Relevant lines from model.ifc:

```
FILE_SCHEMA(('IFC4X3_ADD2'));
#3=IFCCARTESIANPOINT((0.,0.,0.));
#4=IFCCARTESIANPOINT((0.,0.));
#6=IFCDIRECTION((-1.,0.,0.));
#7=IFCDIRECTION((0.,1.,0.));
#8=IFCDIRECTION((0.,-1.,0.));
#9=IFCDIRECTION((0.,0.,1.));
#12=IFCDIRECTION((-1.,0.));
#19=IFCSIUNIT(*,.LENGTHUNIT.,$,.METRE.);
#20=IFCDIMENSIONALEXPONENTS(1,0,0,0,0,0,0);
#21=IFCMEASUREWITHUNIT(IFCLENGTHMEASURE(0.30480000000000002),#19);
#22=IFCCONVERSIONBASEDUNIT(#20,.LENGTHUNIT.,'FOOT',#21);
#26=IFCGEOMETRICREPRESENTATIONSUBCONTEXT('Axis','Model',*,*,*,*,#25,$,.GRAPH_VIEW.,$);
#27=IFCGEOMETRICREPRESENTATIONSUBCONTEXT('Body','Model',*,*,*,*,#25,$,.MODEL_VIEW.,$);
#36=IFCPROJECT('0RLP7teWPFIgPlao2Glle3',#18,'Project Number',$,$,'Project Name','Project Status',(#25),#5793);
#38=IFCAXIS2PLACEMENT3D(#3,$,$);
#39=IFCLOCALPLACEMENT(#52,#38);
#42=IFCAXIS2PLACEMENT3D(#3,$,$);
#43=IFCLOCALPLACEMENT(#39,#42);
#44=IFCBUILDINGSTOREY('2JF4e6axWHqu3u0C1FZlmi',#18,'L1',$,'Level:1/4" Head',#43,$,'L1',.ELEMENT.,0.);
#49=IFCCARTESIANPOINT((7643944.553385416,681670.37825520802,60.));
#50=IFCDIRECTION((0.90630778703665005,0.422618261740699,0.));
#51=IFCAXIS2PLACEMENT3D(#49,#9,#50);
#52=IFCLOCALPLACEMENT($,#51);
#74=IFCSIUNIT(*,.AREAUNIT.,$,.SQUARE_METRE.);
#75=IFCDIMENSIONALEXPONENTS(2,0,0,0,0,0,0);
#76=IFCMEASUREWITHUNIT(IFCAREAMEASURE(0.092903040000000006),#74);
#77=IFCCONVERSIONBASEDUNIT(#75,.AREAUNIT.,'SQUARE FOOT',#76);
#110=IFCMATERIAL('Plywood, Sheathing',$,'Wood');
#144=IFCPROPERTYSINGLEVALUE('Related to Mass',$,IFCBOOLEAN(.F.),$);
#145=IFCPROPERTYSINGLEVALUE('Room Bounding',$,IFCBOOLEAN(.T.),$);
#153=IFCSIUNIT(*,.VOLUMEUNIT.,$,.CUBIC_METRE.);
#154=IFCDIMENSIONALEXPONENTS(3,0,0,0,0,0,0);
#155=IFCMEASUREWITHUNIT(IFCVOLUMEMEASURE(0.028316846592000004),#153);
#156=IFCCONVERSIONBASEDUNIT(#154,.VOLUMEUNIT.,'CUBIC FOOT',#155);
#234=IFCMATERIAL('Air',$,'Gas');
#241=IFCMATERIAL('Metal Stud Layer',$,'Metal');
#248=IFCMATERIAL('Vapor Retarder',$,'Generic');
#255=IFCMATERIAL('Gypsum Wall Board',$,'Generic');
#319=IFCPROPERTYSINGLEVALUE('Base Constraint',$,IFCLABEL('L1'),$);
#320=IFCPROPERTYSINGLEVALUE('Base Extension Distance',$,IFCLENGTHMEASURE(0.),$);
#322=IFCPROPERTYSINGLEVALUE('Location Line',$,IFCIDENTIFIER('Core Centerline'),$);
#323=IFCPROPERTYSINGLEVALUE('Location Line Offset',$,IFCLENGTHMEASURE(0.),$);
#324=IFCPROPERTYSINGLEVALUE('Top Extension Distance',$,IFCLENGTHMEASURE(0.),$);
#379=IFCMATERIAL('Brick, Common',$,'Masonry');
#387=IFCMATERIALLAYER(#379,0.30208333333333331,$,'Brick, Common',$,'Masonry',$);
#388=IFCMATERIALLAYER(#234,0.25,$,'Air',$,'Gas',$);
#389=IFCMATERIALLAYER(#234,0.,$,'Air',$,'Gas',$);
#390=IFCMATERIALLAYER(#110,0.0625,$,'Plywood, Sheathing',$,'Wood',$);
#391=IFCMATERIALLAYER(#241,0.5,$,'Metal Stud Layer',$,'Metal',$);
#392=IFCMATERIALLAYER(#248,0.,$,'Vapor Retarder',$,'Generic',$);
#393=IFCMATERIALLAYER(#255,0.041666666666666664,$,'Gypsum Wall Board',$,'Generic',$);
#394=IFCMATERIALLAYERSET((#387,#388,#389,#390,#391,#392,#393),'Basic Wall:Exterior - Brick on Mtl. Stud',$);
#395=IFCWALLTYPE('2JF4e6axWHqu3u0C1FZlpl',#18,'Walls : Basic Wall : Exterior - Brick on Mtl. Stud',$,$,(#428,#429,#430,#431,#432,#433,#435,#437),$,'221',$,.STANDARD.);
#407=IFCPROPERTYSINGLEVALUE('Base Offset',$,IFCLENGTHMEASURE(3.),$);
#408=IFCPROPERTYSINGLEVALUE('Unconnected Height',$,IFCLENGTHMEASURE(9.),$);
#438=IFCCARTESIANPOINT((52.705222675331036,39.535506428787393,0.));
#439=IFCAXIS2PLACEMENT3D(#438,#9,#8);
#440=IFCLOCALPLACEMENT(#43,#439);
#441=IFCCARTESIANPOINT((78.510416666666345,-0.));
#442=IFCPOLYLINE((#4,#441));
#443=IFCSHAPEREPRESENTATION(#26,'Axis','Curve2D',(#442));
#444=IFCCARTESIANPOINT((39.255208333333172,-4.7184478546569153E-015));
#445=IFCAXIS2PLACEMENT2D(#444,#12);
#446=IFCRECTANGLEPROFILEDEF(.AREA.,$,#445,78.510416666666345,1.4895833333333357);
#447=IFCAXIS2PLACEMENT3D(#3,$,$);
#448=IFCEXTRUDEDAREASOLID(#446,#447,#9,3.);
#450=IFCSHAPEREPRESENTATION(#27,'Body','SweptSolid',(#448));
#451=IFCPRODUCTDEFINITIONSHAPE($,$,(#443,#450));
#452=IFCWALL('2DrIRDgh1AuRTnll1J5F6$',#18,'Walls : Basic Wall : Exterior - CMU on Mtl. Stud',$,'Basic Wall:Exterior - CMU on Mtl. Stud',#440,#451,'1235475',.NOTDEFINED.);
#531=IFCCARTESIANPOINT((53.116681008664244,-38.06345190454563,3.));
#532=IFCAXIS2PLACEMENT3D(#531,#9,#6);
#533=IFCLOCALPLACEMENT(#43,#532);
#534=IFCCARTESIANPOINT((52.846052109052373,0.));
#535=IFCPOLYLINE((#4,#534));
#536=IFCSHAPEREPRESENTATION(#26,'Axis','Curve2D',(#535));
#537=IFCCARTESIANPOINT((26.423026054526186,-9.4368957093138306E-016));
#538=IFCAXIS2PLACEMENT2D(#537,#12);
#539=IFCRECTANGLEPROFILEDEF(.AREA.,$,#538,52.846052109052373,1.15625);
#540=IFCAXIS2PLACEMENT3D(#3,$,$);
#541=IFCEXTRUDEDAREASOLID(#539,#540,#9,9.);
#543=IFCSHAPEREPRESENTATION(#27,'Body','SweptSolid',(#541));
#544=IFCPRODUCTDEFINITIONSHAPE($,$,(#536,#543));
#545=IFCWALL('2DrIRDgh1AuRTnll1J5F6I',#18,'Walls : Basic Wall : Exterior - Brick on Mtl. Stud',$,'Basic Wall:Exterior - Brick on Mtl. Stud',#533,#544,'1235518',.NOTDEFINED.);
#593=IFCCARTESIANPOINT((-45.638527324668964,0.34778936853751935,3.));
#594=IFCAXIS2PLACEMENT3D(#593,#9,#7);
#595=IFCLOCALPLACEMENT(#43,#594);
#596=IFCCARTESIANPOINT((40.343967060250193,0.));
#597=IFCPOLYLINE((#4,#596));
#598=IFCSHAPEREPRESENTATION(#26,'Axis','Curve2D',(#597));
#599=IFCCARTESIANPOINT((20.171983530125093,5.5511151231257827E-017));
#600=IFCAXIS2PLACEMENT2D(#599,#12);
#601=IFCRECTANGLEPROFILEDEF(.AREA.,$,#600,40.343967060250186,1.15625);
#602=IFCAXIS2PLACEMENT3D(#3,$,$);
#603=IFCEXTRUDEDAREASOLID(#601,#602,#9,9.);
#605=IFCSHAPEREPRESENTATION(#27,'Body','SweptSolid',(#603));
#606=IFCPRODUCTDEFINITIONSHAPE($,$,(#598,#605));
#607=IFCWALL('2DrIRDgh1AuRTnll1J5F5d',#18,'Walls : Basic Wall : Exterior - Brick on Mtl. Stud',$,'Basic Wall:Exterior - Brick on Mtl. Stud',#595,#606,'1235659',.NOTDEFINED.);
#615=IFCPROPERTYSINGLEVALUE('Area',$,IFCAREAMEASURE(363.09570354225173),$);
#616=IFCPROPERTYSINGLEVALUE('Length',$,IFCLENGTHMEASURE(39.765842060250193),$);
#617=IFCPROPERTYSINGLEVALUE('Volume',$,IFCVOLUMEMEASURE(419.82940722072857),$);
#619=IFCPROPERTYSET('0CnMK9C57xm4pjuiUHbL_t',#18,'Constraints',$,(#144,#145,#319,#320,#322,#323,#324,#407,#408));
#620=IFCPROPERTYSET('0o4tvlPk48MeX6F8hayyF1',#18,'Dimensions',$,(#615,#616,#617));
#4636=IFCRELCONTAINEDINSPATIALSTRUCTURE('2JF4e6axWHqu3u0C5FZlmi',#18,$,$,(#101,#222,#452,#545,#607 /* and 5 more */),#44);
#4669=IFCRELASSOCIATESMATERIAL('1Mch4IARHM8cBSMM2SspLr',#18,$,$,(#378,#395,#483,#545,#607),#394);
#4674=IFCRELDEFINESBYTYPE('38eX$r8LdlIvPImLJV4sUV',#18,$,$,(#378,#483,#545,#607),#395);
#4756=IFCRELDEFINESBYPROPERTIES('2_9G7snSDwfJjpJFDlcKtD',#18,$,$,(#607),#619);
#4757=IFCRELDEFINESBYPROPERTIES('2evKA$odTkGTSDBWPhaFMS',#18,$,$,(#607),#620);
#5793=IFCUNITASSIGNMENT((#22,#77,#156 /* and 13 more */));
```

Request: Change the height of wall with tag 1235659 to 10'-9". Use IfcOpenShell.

```python
import ifcopenshell
import ifcopenshell.api.pset
import ifcopenshell.geom
import ifcopenshell.util.element
import ifcopenshell.util.representation
import ifcopenshell.util.shape
import ifcopenshell.util.unit

model = ifcopenshell.open("model.ifc")
unit_scale = ifcopenshell.util.unit.calculate_unit_scale(model)
area_scale = ifcopenshell.util.unit.calculate_unit_scale(model, "AREAUNIT")
volume_scale = ifcopenshell.util.unit.calculate_unit_scale(model, "VOLUMEUNIT")
settings = ifcopenshell.geom.settings()


def volume(element):
    """Net volume in cubic metres, openings subtracted."""
    shape = ifcopenshell.geom.create_shape(settings, element)
    return ifcopenshell.util.shape.get_volume(shape.geometry)


wall = model.by_guid("2DrIRDgh1AuRTnll1J5F5d")
before = volume(wall)

body = ifcopenshell.util.representation.get_representation(wall, "Model", "Body")
solid = body.Items[0]
old_height = solid.Depth
solid.Depth = 129 * 0.0254 / unit_scale
after = volume(wall)
thickness = 0.3524  # wall thickness in metres

# Update the stored height, areas and volumes.
pset = model.by_id(ifcopenshell.util.element.get_pset(wall, "Constraints", should_inherit=False)["id"])
ifcopenshell.api.pset.edit_pset(model, pset=pset, properties={
    "Unconnected Height": model.create_entity("IfcLengthMeasure", solid.Depth),
})
pset = model.by_id(ifcopenshell.util.element.get_pset(wall, "Dimensions", should_inherit=False)["id"])
ifcopenshell.api.pset.edit_pset(model, pset=pset, properties={
    "Area": model.create_entity("IfcAreaMeasure", after / thickness / area_scale),
    "Volume": model.create_entity("IfcVolumeMeasure", after / volume_scale),
})

print(f"height {old_height:g} -> {solid.Depth:g}, volume {before:.3f} -> {after:.3f} m3")

model.write("model_v2.ifc")
```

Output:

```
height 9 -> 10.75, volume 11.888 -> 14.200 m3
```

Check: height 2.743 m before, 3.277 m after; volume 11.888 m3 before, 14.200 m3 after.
